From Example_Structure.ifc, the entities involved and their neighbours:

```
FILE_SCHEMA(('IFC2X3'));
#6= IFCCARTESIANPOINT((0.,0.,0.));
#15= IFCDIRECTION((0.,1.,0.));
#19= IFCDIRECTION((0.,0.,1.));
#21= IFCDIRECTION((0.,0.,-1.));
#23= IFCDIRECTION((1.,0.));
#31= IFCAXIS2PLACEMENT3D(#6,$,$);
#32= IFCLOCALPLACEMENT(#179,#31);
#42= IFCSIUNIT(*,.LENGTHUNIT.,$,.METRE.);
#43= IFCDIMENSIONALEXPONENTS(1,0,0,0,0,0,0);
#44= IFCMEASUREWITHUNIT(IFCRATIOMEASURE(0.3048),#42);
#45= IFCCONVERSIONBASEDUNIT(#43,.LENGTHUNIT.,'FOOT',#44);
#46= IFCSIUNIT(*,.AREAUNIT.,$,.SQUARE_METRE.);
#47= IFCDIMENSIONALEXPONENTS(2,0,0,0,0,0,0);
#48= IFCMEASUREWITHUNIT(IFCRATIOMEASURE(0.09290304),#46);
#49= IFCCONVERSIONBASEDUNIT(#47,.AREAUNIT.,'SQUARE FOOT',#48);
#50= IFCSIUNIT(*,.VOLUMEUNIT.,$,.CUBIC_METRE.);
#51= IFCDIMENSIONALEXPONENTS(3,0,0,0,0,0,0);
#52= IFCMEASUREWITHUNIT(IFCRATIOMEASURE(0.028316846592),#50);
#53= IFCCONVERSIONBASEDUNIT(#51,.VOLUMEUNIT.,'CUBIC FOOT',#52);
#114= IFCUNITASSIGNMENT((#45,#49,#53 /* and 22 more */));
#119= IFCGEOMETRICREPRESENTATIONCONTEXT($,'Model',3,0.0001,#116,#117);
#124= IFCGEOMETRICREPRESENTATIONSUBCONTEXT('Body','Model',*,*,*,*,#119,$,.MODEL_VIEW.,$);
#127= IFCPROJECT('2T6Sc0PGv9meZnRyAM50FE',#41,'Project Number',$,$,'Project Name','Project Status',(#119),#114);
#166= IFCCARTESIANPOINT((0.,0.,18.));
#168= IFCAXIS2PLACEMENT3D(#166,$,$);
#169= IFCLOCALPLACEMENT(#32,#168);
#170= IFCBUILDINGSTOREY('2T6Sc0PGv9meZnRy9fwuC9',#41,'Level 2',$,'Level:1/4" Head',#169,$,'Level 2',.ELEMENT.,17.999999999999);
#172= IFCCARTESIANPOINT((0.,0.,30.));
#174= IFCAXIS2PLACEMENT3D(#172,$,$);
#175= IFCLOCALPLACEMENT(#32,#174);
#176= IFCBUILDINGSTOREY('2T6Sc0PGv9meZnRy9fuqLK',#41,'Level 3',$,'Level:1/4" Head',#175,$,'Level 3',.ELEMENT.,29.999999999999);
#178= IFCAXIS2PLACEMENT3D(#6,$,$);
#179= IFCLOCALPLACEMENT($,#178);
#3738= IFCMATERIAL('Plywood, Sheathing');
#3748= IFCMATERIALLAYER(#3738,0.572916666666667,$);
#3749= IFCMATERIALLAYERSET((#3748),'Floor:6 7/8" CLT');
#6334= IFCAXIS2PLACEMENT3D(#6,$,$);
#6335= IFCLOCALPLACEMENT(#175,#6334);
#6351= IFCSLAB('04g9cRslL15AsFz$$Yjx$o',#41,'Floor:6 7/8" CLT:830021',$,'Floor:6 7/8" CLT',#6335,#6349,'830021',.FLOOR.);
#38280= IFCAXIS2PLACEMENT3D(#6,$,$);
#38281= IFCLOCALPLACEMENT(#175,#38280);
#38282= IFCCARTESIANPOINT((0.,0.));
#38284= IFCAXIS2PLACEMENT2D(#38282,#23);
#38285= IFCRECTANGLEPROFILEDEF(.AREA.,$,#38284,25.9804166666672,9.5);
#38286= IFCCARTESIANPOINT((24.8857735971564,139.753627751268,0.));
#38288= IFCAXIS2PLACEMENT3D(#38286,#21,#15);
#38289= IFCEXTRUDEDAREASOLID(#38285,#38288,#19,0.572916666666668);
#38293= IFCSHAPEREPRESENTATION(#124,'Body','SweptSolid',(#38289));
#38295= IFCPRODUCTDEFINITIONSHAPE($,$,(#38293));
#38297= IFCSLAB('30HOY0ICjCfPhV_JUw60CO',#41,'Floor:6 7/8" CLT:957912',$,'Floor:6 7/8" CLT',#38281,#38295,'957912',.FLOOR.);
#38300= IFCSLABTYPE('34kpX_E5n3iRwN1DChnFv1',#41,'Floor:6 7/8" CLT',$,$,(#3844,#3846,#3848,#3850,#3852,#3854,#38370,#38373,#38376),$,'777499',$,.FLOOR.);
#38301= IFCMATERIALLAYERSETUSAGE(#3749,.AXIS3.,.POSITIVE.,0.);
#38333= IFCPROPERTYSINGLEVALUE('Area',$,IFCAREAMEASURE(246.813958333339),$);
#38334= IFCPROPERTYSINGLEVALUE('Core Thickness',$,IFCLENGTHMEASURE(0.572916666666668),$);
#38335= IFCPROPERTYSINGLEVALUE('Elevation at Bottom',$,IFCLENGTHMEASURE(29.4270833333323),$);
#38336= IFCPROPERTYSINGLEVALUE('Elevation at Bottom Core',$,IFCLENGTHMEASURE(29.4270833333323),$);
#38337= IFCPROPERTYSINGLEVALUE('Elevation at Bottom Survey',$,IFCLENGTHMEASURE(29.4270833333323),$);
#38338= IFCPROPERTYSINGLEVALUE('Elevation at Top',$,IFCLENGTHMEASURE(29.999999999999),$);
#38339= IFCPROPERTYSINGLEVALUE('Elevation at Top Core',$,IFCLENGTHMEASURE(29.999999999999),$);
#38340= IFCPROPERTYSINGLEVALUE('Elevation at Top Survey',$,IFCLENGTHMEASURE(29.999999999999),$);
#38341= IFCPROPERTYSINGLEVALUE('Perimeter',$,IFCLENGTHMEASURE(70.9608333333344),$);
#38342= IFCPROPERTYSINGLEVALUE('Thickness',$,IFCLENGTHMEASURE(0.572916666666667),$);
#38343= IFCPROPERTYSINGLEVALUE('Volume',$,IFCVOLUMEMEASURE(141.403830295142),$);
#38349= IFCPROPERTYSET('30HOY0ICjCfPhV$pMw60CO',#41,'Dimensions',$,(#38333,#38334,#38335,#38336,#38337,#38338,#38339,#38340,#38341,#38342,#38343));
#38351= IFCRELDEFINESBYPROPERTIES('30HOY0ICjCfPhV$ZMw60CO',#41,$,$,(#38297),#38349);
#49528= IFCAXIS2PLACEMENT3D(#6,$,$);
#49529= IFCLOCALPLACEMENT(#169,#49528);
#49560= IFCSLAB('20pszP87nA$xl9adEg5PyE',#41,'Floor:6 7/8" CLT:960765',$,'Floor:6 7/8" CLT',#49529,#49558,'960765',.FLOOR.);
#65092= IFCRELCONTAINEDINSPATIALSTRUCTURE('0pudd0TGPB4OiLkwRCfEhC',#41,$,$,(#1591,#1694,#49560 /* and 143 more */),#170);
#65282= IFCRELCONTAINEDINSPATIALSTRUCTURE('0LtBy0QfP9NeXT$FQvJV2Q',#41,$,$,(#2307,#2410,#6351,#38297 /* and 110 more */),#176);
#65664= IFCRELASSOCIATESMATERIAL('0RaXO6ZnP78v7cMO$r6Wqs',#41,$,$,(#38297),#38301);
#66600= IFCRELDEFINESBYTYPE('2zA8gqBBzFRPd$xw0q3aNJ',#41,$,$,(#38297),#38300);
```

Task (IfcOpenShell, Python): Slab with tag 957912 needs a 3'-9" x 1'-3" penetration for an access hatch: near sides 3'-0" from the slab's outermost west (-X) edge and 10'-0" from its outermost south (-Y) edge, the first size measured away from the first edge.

```python
import numpy as np
import ifcopenshell
import ifcopenshell.api.feature
import ifcopenshell.api.geometry
import ifcopenshell.api.pset
import ifcopenshell.api.root
import ifcopenshell.geom
import ifcopenshell.util.element
import ifcopenshell.util.placement
import ifcopenshell.util.representation
import ifcopenshell.util.shape
import ifcopenshell.util.unit

model = ifcopenshell.open("Example_Structure.ifc")
unit_scale = ifcopenshell.util.unit.calculate_unit_scale(model)
area_scale = ifcopenshell.util.unit.calculate_unit_scale(model, "AREAUNIT")
volume_scale = ifcopenshell.util.unit.calculate_unit_scale(model, "VOLUMEUNIT")
settings = ifcopenshell.geom.settings()


def volume(element):
    """Net volume in cubic metres, openings subtracted."""
    shape = ifcopenshell.geom.create_shape(settings, element)
    return ifcopenshell.util.shape.get_volume(shape.geometry)


slab = model.by_guid("30HOY0ICjCfPhV_JUw60CO")
before = volume(slab)

# Extent in the slab's own axes, in metres. The edges named are its -X and -Y sides.
slab_shape = ifcopenshell.geom.create_shape(settings, slab)
vertices = ifcopenshell.util.shape.get_vertices(slab_shape.geometry)
x_min, y_min, bottom = vertices.min(axis=0)
top = vertices[:, 2].max()

opening = ifcopenshell.api.root.create_entity(model, ifc_class="IfcOpeningElement", name="Access hatch opening")
context = ifcopenshell.util.representation.get_context(model, "Model", "Body", "MODEL_VIEW")
width, depth = 1.143, 0.381
outline = [(0.0, 0.0), (width, 0.0), (width, depth), (0.0, depth), (0.0, 0.0)]
# Overshoot both faces by 50 mm so the cut is clean.
shape = ifcopenshell.api.geometry.add_slab_representation(
    model, context=context, depth=top - bottom + 0.1, polyline=outline
)
ifcopenshell.api.geometry.assign_representation(model, product=opening, representation=shape)

matrix = ifcopenshell.util.placement.get_local_placement(slab.ObjectPlacement)
matrix[:, 3] = matrix @ np.append(np.array([x_min + 0.9144, y_min + 3.048, bottom - 0.05]) / unit_scale, 1.0)
ifcopenshell.api.geometry.edit_object_placement(model, product=opening, matrix=matrix, is_si=False)
ifcopenshell.api.feature.add_feature(model, feature=opening, element=slab)

after = volume(slab)

# Update the slab's stored quantities.
pset = model.by_id(ifcopenshell.util.element.get_pset(slab, "Dimensions", should_inherit=False)["id"])
ifcopenshell.api.pset.edit_pset(model, pset=pset, properties={
    "Area": model.create_entity("IfcAreaMeasure", after / (top - bottom) / area_scale),
    "Volume": model.create_entity("IfcVolumeMeasure", after / volume_scale),
})

print(f"slab volume {before:.3f} -> {after:.3f} m3")

model.write("Example_Structure_v2.ifc")
```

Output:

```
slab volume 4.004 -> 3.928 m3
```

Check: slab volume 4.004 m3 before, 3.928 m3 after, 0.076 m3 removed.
